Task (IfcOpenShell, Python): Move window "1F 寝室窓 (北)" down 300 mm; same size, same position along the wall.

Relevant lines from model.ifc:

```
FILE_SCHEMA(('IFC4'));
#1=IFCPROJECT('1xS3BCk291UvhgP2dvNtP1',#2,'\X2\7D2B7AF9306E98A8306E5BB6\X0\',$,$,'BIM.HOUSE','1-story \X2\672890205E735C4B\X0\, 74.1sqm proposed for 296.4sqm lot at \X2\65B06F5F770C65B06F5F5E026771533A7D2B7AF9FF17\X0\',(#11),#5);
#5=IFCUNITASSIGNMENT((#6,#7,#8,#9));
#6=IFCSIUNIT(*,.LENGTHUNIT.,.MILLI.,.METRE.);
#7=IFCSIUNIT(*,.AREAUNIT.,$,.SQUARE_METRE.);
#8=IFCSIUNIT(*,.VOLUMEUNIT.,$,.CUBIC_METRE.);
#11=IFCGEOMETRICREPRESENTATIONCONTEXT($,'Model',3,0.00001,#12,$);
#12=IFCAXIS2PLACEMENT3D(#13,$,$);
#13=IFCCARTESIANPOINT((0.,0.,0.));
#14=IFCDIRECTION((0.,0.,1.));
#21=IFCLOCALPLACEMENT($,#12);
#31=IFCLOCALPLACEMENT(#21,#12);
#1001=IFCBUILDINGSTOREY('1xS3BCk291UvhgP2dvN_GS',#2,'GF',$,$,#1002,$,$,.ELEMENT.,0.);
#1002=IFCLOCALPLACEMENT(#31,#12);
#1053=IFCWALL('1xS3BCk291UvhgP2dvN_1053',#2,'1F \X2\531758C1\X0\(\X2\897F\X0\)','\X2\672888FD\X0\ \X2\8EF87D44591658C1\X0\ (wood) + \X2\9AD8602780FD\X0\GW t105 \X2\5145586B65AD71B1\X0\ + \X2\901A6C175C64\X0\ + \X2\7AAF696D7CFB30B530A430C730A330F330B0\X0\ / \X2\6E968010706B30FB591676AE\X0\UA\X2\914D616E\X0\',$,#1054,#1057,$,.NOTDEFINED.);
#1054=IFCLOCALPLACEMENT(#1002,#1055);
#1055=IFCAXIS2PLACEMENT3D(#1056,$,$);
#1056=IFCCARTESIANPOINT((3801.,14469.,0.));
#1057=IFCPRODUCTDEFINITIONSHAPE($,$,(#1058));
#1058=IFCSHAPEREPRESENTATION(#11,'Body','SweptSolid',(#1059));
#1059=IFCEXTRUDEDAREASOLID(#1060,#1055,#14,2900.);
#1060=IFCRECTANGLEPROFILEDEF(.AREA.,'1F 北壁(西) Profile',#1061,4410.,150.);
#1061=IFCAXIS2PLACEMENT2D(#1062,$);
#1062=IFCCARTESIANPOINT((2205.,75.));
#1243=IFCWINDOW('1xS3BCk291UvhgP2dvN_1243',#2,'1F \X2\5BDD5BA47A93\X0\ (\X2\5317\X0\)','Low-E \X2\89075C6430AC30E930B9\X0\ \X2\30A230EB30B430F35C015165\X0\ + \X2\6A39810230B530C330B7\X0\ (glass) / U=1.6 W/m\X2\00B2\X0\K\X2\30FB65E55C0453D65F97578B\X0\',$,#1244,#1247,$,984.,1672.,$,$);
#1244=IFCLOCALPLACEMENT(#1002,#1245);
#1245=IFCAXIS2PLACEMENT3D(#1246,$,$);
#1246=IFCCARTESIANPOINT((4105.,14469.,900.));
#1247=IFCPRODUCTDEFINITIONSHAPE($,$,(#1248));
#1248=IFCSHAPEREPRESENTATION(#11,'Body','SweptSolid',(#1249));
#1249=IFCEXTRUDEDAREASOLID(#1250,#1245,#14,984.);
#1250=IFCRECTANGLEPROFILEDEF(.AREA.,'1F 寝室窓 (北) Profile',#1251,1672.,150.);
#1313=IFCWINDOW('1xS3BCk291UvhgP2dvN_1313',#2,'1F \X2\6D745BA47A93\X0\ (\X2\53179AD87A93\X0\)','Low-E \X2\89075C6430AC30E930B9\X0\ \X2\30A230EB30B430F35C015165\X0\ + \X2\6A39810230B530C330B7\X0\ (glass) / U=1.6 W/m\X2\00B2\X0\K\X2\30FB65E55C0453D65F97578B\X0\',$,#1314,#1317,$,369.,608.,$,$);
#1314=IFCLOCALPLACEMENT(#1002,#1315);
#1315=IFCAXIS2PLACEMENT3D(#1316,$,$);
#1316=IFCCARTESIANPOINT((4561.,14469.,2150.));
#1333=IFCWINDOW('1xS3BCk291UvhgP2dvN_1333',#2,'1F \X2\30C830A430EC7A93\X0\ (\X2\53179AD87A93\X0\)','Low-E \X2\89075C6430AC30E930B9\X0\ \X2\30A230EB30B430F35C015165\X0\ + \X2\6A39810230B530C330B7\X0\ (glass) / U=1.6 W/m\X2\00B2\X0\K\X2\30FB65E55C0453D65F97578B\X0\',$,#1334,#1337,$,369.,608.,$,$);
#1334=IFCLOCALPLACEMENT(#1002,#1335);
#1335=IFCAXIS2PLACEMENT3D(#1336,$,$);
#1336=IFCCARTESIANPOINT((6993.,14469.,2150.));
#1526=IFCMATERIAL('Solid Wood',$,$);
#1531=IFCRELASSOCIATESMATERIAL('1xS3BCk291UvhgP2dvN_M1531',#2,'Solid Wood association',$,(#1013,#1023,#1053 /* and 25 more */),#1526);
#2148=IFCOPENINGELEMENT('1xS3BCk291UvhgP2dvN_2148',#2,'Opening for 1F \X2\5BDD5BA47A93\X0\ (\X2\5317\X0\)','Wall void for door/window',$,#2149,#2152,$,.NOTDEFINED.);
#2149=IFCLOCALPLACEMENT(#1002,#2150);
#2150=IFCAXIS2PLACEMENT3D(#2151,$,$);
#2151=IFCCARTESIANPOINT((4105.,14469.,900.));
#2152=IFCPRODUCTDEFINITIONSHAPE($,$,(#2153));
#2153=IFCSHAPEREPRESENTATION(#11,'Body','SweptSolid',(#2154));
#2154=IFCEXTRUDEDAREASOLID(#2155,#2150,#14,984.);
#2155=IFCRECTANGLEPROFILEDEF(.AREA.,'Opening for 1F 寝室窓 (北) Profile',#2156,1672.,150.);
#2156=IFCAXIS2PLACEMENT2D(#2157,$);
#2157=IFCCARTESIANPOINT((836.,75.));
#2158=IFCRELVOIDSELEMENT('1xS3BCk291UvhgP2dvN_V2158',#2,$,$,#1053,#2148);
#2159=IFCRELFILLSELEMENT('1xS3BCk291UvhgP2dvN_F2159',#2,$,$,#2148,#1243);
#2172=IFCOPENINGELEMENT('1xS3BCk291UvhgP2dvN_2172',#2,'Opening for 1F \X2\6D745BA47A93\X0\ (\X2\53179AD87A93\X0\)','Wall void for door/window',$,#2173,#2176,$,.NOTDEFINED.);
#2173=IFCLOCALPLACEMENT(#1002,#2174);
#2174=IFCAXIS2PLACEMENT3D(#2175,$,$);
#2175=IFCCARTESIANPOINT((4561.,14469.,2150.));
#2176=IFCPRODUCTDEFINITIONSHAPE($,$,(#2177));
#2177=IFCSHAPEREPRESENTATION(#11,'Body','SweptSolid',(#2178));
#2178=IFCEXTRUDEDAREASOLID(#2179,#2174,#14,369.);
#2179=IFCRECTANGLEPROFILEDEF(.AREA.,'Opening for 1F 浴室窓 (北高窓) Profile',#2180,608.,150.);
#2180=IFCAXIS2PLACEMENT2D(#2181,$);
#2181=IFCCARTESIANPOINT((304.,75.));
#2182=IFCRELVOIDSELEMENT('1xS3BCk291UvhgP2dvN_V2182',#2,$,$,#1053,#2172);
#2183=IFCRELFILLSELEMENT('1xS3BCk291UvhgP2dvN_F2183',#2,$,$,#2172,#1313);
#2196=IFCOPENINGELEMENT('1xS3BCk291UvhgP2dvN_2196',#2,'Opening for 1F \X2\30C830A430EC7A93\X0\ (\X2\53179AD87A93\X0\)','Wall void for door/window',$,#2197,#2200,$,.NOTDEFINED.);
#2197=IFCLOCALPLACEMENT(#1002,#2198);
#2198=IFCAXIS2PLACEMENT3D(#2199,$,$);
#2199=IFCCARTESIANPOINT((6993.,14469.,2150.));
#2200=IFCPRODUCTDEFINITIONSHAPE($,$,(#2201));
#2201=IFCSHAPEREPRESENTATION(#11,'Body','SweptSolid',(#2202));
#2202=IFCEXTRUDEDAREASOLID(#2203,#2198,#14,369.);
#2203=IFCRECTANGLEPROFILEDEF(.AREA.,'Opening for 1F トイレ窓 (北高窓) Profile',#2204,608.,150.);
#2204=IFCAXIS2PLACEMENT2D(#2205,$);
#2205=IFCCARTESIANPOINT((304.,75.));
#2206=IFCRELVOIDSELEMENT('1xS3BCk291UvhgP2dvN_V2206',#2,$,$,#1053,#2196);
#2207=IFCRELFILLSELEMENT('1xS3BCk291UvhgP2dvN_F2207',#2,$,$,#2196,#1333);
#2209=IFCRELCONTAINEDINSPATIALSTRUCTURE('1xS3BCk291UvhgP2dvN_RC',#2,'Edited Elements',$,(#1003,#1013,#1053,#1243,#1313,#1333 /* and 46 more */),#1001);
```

```python
import numpy as np
import ifcopenshell
import ifcopenshell.api.geometry
import ifcopenshell.util.placement
import ifcopenshell.util.unit

model = ifcopenshell.open("model.ifc")
unit_scale = ifcopenshell.util.unit.calculate_unit_scale(model)

window = model.by_id(1243)
opening = window.FillsVoids[0].RelatingOpeningElement
dz = -0.3 / unit_scale

shift = np.array([0.0, 0.0, dz])
# The window is not placed relative to its opening, so move both.
for product in (opening, window):
    matrix = ifcopenshell.util.placement.get_local_placement(product.ObjectPlacement)
    matrix[:3, 3] += shift
    ifcopenshell.api.geometry.edit_object_placement(model, product=product, matrix=matrix, is_si=False)

print(f"moved by {dz * unit_scale:+.3f} m")

model.write("model-out.ifc")
```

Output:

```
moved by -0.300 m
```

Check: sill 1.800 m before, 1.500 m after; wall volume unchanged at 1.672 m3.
